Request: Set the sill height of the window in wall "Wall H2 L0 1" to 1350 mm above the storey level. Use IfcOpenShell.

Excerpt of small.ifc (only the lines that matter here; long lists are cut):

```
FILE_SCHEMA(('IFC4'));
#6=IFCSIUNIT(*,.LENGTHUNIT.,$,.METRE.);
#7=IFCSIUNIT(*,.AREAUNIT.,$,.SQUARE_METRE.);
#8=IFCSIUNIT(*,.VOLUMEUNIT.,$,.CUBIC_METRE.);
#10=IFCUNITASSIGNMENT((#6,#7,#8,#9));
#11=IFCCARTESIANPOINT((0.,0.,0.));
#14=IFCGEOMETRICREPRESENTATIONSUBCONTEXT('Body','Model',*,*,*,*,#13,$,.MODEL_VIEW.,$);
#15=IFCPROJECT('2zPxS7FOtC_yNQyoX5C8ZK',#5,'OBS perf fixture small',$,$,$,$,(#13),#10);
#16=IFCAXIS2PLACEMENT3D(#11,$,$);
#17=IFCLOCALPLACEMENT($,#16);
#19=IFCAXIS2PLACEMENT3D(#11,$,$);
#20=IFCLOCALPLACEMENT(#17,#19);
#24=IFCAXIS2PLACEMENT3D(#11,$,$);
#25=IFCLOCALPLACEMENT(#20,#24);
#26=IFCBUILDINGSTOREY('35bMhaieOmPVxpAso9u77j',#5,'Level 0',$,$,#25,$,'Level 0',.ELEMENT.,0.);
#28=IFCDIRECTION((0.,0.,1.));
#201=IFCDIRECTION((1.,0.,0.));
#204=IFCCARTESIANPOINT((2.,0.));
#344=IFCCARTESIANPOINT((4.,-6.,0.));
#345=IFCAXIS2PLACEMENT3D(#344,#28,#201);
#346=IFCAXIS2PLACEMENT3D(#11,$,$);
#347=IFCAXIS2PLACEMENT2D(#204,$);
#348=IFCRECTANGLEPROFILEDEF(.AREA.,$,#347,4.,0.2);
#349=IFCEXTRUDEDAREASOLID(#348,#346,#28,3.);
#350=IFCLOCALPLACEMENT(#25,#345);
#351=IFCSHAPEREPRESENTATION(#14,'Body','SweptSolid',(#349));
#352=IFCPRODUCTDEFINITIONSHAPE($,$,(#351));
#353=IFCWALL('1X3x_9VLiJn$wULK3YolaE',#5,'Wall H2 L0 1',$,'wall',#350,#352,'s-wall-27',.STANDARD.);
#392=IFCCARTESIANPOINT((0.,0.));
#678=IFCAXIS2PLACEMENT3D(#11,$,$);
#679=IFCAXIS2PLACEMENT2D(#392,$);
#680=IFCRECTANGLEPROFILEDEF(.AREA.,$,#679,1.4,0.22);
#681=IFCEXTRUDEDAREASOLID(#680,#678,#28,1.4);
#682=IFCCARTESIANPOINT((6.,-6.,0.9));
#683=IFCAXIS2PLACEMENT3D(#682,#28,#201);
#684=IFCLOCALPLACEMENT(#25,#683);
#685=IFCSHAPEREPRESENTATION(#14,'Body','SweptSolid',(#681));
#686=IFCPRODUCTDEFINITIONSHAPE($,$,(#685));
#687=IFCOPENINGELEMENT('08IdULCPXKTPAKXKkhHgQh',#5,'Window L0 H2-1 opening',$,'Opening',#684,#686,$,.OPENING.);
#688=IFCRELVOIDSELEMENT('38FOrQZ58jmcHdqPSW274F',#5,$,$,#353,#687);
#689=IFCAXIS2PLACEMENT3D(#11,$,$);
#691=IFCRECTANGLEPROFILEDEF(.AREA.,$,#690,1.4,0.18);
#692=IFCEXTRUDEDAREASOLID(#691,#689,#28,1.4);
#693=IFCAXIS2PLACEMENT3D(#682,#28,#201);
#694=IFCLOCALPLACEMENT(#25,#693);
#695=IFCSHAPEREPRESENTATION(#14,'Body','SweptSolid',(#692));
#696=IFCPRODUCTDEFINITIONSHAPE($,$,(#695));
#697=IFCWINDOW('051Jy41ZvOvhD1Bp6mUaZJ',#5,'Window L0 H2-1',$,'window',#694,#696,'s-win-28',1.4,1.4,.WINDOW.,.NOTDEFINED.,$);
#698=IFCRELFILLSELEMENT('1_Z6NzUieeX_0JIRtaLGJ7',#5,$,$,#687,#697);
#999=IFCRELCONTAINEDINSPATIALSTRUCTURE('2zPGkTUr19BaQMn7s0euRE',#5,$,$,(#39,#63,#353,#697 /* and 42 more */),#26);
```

```python
import numpy as np
import ifcopenshell
import ifcopenshell.api.geometry
import ifcopenshell.geom
import ifcopenshell.util.element
import ifcopenshell.util.placement
import ifcopenshell.util.shape
import ifcopenshell.util.unit

model = ifcopenshell.open("small.ifc")
unit_scale = ifcopenshell.util.unit.calculate_unit_scale(model)

window = model.by_guid("051Jy41ZvOvhD1Bp6mUaZJ")
opening = window.FillsVoids[0].RelatingOpeningElement
storey = ifcopenshell.util.element.get_container(window, ifc_class="IfcBuildingStorey")
level = ifcopenshell.util.placement.get_local_placement(storey.ObjectPlacement)[2, 3]

# The opening's origin need not be at the sill, so measure its lowest point.
shape = ifcopenshell.geom.create_shape(ifcopenshell.geom.settings(), opening)
bottom = ifcopenshell.util.shape.get_shape_bottom_elevation(shape, shape.geometry) / unit_scale
dz = level + 1.35 / unit_scale - bottom

shift = np.array([0.0, 0.0, dz])
# The window is not placed relative to its opening, so move both.
for product in (opening, window):
    matrix = ifcopenshell.util.placement.get_local_placement(product.ObjectPlacement)
    matrix[:3, 3] += shift
    ifcopenshell.api.geometry.edit_object_placement(model, product=product, matrix=matrix, is_si=False)

print(f"moved by {dz * unit_scale:+.3f} m")

model.write("small-out.ifc")
```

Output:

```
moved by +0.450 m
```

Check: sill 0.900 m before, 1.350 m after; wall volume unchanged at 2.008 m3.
